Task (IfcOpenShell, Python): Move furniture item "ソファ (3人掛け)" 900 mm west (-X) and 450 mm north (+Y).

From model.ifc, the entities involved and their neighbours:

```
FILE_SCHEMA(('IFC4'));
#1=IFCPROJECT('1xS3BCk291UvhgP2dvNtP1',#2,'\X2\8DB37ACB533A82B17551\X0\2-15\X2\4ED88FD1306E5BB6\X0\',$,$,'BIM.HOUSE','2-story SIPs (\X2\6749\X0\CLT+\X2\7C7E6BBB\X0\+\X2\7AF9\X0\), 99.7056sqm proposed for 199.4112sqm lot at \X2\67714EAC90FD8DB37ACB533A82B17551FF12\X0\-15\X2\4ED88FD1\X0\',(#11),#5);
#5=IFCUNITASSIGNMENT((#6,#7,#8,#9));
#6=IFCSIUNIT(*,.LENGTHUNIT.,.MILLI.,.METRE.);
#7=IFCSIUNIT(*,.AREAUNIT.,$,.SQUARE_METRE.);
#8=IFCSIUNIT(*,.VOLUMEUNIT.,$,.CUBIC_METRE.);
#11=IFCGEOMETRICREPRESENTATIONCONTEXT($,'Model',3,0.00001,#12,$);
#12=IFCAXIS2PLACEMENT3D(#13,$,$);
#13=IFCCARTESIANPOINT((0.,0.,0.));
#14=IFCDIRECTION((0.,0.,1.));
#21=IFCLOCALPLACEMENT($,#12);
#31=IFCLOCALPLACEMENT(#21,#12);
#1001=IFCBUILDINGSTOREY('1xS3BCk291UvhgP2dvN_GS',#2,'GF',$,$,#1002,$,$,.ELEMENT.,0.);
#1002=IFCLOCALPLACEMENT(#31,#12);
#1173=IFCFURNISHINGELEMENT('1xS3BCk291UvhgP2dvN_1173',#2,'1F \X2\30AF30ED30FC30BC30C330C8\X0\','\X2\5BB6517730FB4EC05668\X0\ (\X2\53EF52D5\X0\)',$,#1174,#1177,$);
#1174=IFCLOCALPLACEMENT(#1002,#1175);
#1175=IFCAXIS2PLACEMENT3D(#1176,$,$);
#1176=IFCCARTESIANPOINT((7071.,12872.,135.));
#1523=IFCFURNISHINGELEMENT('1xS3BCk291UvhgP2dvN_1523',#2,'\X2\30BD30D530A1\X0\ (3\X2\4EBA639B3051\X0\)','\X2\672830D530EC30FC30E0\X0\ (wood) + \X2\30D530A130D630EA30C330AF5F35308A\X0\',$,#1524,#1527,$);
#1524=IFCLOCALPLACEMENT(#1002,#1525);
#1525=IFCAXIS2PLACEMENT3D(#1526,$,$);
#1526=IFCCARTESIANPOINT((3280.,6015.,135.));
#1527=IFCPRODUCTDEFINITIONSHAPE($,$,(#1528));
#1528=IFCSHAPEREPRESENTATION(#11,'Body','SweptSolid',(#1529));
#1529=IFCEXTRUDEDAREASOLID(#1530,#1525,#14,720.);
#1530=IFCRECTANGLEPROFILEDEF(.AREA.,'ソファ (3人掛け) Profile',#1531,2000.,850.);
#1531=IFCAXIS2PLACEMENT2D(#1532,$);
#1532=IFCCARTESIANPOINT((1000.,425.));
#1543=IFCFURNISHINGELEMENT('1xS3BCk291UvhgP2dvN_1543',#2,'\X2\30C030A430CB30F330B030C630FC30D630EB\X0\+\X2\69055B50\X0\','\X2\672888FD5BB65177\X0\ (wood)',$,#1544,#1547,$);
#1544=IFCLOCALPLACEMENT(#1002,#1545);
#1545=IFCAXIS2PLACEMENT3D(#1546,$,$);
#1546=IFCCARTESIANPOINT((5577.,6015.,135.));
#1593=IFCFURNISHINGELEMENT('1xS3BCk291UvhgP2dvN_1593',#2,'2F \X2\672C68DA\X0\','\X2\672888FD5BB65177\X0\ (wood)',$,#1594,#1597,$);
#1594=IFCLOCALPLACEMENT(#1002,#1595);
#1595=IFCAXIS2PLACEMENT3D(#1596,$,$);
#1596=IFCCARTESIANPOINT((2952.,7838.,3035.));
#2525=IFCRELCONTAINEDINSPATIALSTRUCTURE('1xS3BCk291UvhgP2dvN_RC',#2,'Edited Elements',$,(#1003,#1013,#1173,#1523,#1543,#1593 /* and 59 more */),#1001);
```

```python
import ifcopenshell
import ifcopenshell.api.geometry
import ifcopenshell.util.placement
import ifcopenshell.util.unit

model = ifcopenshell.open("model.ifc")
unit_scale = ifcopenshell.util.unit.calculate_unit_scale(model)

item = model.by_guid("1xS3BCk291UvhgP2dvN_1523")
matrix = ifcopenshell.util.placement.get_local_placement(item.ObjectPlacement)
matrix[0, 3] -= 0.9 / unit_scale
matrix[1, 3] += 0.45 / unit_scale
ifcopenshell.api.geometry.edit_object_placement(model, product=item, matrix=matrix, is_si=False)

print(ifcopenshell.util.placement.get_local_placement(item.ObjectPlacement).round(3) + 0.0)

model.write("model_v2.ifc")
```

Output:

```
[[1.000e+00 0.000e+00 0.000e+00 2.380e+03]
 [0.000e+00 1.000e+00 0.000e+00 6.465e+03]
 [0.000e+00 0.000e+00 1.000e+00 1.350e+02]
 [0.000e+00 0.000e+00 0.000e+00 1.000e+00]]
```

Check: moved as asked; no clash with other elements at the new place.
